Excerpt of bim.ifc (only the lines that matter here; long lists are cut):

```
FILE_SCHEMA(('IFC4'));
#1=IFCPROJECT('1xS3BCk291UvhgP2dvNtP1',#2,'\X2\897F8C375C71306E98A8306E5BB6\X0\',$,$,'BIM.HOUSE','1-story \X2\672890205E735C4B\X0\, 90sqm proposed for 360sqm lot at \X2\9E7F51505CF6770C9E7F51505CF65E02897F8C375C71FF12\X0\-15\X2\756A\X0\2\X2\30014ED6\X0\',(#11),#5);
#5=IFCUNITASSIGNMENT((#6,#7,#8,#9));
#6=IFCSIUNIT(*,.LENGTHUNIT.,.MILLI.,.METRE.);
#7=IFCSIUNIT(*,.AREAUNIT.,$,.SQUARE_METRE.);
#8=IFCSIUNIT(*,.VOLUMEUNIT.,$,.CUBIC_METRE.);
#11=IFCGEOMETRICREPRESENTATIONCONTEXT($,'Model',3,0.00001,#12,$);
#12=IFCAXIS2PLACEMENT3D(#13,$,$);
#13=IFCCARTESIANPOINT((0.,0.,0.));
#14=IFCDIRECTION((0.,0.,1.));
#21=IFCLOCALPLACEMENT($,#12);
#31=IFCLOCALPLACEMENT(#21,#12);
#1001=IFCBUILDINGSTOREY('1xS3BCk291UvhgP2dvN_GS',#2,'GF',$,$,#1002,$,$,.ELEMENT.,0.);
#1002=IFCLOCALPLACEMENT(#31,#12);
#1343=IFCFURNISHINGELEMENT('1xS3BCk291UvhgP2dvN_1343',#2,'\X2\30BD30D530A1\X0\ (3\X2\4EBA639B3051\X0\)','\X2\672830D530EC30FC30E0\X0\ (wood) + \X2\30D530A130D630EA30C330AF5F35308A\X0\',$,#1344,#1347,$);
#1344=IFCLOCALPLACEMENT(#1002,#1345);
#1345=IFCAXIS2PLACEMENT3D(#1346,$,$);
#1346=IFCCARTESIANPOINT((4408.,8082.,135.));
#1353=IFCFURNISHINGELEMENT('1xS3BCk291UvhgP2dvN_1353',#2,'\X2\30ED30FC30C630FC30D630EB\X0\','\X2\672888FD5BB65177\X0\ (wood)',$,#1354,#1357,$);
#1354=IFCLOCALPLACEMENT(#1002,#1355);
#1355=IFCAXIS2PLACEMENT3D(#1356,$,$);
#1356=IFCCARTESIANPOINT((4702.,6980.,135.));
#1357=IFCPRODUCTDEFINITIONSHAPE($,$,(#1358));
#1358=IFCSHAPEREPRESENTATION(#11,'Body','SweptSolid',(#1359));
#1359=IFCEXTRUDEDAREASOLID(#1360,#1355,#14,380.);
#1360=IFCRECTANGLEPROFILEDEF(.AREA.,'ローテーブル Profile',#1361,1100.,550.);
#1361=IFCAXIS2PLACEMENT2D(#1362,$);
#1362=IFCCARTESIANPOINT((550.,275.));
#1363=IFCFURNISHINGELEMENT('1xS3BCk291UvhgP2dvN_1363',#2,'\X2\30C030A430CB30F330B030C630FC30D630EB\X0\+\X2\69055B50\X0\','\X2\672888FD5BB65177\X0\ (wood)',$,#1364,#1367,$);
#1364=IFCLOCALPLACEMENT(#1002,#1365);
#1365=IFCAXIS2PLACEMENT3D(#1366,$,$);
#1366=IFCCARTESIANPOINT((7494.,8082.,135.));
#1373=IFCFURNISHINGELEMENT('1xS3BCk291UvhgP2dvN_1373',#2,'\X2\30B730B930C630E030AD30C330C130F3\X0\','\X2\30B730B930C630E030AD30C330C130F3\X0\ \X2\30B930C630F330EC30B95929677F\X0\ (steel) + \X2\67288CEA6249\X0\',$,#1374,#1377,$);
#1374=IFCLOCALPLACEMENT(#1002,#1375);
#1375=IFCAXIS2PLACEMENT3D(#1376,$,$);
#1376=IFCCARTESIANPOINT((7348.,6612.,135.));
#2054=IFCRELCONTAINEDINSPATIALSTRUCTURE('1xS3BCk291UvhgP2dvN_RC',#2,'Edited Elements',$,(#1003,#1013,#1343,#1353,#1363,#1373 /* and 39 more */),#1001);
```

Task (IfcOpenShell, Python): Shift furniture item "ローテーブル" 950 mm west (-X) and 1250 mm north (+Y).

```python
import ifcopenshell
import ifcopenshell.api.geometry
import ifcopenshell.util.placement

model = ifcopenshell.open("bim.ifc")

item = model.by_guid("1xS3BCk291UvhgP2dvN_1353")
matrix = ifcopenshell.util.placement.get_local_placement(item.ObjectPlacement)
matrix[0, 3] -= 950.0
matrix[1, 3] += 1250.0
ifcopenshell.api.geometry.edit_object_placement(model, product=item, matrix=matrix, is_si=False)

print(ifcopenshell.util.placement.get_local_placement(item.ObjectPlacement).round(3) + 0.0)

model.write("bim_v2.ifc")
```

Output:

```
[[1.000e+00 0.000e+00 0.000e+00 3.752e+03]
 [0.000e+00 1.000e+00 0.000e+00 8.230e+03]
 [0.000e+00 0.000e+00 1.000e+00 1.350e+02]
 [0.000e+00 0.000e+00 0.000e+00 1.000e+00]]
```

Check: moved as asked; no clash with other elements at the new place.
